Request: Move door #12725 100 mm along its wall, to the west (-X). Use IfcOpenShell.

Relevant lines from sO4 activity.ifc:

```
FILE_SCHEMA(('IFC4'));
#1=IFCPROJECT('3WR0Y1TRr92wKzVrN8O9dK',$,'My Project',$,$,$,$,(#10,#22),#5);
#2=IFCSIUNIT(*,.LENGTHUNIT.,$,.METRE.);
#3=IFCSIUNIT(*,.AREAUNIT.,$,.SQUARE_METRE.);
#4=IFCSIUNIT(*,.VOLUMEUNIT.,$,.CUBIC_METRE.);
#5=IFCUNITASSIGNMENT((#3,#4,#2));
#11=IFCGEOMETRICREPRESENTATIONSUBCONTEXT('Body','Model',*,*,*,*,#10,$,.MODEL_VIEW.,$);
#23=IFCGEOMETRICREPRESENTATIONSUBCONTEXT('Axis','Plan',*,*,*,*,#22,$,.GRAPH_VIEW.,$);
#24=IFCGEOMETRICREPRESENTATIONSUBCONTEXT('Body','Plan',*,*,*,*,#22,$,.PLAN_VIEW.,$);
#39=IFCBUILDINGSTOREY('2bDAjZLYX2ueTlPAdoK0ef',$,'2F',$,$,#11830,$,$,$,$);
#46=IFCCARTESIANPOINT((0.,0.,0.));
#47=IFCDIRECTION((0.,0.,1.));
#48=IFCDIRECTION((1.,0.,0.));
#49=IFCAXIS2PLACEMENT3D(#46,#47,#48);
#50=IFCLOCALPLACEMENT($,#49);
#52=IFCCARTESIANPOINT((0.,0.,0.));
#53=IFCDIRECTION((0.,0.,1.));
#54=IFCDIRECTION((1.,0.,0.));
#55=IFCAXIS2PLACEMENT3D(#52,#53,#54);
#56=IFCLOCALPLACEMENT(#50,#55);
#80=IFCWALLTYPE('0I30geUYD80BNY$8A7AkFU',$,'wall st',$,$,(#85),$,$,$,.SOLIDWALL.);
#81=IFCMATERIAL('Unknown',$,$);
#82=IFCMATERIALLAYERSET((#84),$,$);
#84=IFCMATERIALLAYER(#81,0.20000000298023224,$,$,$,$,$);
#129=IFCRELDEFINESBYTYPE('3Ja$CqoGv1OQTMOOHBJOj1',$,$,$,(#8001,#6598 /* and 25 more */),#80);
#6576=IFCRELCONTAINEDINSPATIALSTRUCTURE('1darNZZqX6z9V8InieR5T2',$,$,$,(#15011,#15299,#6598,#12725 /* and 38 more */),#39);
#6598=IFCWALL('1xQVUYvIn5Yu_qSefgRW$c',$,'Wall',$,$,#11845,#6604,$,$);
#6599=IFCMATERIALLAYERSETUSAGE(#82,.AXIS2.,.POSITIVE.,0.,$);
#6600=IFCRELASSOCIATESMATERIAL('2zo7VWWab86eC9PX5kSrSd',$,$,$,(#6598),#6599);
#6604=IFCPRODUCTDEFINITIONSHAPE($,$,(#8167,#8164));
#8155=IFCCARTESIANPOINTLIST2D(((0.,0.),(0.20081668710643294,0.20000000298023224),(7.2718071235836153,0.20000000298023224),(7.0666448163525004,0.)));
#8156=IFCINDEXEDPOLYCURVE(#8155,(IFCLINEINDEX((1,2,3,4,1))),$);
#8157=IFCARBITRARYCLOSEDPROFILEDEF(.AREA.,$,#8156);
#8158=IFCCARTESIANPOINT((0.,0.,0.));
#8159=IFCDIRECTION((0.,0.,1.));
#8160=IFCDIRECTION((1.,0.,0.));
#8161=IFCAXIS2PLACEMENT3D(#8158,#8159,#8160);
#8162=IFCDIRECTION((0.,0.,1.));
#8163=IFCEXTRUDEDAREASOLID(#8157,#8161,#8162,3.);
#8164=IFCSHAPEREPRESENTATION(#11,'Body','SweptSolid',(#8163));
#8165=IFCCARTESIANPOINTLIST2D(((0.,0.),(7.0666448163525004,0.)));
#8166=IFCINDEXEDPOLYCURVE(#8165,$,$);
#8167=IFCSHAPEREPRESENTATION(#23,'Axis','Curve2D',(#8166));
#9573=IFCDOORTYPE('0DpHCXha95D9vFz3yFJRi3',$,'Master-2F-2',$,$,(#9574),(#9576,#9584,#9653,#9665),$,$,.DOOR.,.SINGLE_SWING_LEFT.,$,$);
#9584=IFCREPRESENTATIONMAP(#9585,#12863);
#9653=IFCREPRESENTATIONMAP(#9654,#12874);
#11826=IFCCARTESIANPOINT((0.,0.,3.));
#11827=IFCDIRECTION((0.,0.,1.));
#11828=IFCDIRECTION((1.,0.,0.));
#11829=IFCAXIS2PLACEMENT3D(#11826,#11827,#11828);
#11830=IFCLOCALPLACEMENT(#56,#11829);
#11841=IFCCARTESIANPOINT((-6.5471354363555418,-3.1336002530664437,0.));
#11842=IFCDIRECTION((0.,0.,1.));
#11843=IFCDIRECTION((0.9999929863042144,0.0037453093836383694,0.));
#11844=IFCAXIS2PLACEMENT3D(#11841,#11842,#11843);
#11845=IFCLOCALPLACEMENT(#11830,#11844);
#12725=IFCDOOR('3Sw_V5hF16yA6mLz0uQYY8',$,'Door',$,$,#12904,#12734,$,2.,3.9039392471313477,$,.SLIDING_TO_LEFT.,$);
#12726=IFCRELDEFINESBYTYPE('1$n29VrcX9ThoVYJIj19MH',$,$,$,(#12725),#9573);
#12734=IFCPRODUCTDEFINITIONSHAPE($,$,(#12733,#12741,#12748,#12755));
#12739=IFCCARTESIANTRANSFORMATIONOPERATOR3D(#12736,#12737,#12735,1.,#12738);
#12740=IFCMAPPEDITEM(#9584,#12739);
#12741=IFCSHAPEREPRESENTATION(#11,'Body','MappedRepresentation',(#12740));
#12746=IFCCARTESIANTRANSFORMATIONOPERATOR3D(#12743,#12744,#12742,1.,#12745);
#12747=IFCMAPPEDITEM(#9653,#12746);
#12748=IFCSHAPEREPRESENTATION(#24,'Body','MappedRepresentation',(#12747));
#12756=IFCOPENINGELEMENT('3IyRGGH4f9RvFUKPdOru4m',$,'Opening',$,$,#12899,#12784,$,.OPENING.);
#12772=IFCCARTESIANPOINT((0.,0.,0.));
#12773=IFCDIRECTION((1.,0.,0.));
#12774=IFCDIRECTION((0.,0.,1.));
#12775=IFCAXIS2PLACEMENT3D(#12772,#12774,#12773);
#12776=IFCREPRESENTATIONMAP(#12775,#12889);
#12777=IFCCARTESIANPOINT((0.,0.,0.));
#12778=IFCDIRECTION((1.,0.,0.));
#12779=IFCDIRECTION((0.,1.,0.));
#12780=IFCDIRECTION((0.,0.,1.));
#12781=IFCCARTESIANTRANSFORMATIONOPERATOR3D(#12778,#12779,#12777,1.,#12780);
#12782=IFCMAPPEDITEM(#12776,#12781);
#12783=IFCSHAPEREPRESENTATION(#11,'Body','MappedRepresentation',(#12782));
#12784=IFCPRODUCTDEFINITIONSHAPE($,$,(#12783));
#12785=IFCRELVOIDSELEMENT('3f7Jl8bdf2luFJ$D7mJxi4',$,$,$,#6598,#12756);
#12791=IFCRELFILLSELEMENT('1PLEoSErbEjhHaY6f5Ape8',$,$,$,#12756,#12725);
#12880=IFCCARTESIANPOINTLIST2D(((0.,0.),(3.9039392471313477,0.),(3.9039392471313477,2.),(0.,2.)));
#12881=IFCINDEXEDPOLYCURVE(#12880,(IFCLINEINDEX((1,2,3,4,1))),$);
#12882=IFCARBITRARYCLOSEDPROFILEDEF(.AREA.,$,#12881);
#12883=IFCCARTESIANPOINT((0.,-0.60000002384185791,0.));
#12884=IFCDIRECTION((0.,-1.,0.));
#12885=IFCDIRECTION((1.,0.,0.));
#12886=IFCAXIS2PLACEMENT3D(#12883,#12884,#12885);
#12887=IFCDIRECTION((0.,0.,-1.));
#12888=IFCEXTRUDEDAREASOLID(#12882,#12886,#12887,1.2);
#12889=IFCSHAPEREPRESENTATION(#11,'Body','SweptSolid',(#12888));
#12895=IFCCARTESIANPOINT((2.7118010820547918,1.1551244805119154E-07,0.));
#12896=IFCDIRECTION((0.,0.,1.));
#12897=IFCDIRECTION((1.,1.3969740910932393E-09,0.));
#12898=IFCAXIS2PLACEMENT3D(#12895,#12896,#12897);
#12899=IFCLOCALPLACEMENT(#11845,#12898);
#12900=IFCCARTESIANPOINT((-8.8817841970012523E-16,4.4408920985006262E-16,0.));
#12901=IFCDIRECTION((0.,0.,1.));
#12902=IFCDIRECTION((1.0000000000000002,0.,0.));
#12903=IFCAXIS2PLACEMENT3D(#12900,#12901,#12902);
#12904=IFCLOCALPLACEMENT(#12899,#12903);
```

```python
import ifcopenshell
import ifcopenshell.api.geometry
import ifcopenshell.util.placement
import ifcopenshell.util.unit

model = ifcopenshell.open("sO4 activity.ifc")
unit_scale = ifcopenshell.util.unit.calculate_unit_scale(model)

door = model.by_guid("3Sw_V5hF16yA6mLz0uQYY8")
opening = door.FillsVoids[0].RelatingOpeningElement
wall = opening.VoidsElements[0].RelatingBuildingElement

wall_matrix = ifcopenshell.util.placement.get_local_placement(wall.ObjectPlacement)
shift = wall_matrix[:3, 0] * -0.1 / unit_scale
before = ifcopenshell.util.placement.get_local_placement(door.ObjectPlacement)[:3, 3].copy()

# The door is placed relative to its opening, so it follows when the opening moves.
matrix = ifcopenshell.util.placement.get_local_placement(opening.ObjectPlacement)
matrix[:3, 3] += shift
ifcopenshell.api.geometry.edit_object_placement(
    model, product=opening, matrix=matrix, is_si=False, should_transform_children=True
)

after = ifcopenshell.util.placement.get_local_placement(door.ObjectPlacement)[:3, 3]
print("door moved by", (after - before).round(3) + 0.0)

model.write("sO4 activity-out.ifc")
```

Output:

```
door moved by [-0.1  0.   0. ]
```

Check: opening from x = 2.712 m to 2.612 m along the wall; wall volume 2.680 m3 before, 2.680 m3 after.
